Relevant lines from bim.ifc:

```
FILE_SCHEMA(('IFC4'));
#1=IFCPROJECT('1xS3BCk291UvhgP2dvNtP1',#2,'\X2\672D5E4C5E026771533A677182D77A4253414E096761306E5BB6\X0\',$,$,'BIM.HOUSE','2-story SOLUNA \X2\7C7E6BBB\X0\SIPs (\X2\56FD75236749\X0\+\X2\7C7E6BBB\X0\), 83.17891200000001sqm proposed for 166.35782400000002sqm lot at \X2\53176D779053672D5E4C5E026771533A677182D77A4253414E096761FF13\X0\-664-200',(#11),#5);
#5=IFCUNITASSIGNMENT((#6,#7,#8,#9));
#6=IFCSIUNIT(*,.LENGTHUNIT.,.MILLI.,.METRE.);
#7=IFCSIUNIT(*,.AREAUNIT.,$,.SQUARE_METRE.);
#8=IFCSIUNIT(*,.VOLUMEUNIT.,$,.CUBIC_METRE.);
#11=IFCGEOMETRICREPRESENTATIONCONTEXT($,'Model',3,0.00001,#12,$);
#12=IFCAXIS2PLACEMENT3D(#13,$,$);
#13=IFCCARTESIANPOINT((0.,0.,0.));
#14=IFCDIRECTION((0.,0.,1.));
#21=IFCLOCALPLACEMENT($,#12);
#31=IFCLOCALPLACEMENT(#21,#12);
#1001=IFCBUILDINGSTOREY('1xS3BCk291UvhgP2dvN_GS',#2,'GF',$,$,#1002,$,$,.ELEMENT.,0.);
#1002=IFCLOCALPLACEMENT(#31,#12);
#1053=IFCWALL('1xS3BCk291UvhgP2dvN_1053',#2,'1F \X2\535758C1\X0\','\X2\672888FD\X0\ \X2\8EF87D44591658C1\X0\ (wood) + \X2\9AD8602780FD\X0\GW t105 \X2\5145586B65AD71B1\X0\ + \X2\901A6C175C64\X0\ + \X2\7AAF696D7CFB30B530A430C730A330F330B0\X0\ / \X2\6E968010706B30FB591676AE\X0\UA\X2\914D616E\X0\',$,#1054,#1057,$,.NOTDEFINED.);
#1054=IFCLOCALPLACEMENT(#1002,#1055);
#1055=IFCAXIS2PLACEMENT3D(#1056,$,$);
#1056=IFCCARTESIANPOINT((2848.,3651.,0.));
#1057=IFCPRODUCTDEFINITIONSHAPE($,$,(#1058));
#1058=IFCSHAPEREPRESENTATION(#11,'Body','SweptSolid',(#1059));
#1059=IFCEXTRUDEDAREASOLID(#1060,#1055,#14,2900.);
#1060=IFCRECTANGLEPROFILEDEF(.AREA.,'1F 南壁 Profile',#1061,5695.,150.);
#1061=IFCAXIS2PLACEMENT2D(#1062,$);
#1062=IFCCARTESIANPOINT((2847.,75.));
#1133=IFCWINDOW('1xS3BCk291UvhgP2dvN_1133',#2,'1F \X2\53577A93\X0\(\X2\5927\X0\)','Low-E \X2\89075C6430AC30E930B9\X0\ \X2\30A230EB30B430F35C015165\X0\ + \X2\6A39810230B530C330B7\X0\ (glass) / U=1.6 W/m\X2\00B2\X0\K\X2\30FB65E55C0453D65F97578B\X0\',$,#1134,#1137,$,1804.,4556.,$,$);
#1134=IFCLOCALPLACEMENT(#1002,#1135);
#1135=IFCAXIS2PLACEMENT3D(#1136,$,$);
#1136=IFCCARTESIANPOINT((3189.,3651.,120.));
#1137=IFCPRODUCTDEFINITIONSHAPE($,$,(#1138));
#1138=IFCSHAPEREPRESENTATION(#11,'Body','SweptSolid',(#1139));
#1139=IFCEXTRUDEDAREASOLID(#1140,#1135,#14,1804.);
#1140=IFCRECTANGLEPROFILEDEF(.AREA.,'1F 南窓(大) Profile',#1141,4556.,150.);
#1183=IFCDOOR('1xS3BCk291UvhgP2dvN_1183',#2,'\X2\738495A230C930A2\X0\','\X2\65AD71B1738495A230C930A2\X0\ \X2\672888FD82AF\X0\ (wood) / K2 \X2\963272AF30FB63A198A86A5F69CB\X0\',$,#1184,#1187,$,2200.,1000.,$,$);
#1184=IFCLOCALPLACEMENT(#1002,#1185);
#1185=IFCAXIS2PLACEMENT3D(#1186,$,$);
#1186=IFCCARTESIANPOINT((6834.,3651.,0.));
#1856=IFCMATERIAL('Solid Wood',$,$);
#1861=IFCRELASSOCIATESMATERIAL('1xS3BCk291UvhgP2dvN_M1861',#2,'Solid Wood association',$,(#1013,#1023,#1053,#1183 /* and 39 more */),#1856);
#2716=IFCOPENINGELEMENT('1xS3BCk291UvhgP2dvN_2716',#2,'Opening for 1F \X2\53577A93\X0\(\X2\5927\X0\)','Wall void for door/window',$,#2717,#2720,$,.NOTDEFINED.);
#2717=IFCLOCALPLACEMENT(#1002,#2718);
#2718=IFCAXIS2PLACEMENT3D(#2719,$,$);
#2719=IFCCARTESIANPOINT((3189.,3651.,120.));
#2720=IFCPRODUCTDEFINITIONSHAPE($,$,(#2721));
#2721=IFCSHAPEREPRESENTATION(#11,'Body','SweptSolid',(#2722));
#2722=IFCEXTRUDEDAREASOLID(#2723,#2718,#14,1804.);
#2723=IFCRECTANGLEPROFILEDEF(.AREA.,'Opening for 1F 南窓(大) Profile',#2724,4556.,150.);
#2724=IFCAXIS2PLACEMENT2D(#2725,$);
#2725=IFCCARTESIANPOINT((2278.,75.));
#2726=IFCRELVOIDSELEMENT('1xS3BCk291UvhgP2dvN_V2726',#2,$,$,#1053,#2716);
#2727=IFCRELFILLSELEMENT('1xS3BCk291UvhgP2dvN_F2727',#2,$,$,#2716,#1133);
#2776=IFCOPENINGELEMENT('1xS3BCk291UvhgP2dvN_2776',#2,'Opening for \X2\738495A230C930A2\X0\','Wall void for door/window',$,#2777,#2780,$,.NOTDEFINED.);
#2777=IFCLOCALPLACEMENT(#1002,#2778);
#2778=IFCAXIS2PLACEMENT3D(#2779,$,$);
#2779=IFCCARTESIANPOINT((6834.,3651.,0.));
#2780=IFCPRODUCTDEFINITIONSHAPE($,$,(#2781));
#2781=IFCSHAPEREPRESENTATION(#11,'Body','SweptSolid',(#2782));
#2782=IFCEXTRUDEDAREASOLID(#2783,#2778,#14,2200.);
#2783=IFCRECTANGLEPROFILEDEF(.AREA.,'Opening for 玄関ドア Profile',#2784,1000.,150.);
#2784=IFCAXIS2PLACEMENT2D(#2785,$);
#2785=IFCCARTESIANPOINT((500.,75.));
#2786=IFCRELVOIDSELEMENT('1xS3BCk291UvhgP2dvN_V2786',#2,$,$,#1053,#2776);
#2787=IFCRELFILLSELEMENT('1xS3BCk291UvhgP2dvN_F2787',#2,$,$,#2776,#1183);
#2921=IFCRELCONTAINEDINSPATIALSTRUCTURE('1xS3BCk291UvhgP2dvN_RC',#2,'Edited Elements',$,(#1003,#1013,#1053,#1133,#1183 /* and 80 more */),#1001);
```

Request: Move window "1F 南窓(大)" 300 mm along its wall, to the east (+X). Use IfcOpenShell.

```python
import ifcopenshell
import ifcopenshell.api.geometry
import ifcopenshell.util.placement
import ifcopenshell.util.unit

model = ifcopenshell.open("bim.ifc")
unit_scale = ifcopenshell.util.unit.calculate_unit_scale(model)

window = model.by_id(1133)
opening = window.FillsVoids[0].RelatingOpeningElement
wall = opening.VoidsElements[0].RelatingBuildingElement

wall_matrix = ifcopenshell.util.placement.get_local_placement(wall.ObjectPlacement)
shift = wall_matrix[:3, 0] * 0.3 / unit_scale
before = ifcopenshell.util.placement.get_local_placement(window.ObjectPlacement)[:3, 3].copy()

# The window is not placed relative to its opening, so move both.
for product in (opening, window):
    matrix = ifcopenshell.util.placement.get_local_placement(product.ObjectPlacement)
    matrix[:3, 3] += shift
    ifcopenshell.api.geometry.edit_object_placement(model, product=product, matrix=matrix, is_si=False)

after = ifcopenshell.util.placement.get_local_placement(window.ObjectPlacement)[:3, 3]
print("window moved by", (after - before).round(3) + 0.0)

model.write("bim-out.ifc")
```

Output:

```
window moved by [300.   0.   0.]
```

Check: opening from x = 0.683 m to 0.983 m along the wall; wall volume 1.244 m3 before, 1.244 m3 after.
